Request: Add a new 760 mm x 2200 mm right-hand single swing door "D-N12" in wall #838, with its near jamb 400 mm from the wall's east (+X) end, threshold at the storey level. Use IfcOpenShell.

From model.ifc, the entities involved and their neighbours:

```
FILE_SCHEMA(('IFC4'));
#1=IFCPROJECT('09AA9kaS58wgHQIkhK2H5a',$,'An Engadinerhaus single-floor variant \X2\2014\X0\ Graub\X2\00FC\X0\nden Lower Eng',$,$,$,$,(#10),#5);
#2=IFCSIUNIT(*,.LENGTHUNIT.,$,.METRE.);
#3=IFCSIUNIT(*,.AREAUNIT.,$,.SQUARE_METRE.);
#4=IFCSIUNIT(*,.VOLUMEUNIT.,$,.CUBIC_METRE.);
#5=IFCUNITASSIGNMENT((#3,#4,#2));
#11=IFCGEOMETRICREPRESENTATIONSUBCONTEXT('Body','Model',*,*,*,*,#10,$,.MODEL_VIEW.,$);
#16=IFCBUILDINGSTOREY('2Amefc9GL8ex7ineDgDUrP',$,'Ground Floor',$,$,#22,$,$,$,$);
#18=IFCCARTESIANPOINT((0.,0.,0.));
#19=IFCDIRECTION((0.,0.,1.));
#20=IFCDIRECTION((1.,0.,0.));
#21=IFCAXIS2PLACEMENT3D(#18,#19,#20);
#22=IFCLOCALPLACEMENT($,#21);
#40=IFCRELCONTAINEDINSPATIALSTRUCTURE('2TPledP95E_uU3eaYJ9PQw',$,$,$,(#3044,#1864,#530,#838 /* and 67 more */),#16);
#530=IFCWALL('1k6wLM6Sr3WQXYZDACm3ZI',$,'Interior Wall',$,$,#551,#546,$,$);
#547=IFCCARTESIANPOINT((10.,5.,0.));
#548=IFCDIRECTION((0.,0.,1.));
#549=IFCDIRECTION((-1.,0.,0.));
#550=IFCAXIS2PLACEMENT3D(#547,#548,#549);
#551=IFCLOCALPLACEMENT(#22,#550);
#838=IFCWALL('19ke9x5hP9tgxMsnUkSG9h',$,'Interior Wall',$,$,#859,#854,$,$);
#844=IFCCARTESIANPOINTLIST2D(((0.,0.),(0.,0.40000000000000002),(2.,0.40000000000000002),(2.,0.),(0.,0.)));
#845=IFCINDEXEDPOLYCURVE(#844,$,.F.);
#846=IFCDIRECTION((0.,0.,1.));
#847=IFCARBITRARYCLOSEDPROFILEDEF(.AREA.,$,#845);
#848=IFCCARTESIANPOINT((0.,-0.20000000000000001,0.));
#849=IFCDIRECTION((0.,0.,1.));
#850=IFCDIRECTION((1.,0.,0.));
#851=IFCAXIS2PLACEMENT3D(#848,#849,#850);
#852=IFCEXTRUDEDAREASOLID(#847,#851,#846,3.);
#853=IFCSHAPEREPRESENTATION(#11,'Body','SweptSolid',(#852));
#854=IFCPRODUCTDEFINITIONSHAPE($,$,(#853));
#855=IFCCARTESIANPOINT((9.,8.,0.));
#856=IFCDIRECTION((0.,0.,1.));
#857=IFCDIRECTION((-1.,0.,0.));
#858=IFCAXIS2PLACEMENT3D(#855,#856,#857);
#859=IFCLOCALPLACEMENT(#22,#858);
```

```python
import numpy as np
import ifcopenshell
import ifcopenshell.api.feature
import ifcopenshell.api.geometry
import ifcopenshell.api.root
import ifcopenshell.api.spatial
import ifcopenshell.geom
import ifcopenshell.util.element
import ifcopenshell.util.placement
import ifcopenshell.util.representation
import ifcopenshell.util.shape
import ifcopenshell.util.unit

model = ifcopenshell.open("model.ifc")
unit_scale = ifcopenshell.util.unit.calculate_unit_scale(model)
settings = ifcopenshell.geom.settings()


def volume(element):
    """Net volume in cubic metres, openings subtracted."""
    shape = ifcopenshell.geom.create_shape(settings, element)
    return ifcopenshell.util.shape.get_volume(shape.geometry)


wall = model.by_guid("19ke9x5hP9tgxMsnUkSG9h")
storey = ifcopenshell.util.element.get_container(wall, ifc_class="IfcBuildingStorey")
context = ifcopenshell.util.representation.get_context(model, "Model", "Body", "MODEL_VIEW")
before = volume(wall)

width, height, from_end, sill = 0.76, 2.2, 0.4, 0.0  # metres

# The wall runs along its own X axis, and the end named is its -X end.
wall_shape = ifcopenshell.geom.create_shape(settings, wall)
x, y, z = ifcopenshell.util.shape.get_vertices(wall_shape.geometry).T
start = x.min() + from_end
face, thickness = float(y.min()), float(y.max() - y.min())
wall_matrix = ifcopenshell.util.placement.get_local_placement(wall.ObjectPlacement)
level = ifcopenshell.util.placement.get_local_placement(storey.ObjectPlacement)[2, 3]


def in_wall(x, y):
    """Placement at x, y metres in the wall's axes, at sill height."""
    matrix = wall_matrix.copy()
    matrix[:, 3] = wall_matrix @ np.array([x / unit_scale, y / unit_scale, 0.0, 1.0])
    matrix[2, 3] = level + sill / unit_scale
    return matrix


# Opening: a box that overshoots both wall faces by 50 mm.
opening = ifcopenshell.api.root.create_entity(model, ifc_class="IfcOpeningElement", predefined_type="OPENING")
box = ifcopenshell.api.geometry.add_wall_representation(
    model, context=context, length=width, height=height, thickness=thickness + 0.1
)
ifcopenshell.api.geometry.assign_representation(model, product=opening, representation=box)
ifcopenshell.api.geometry.edit_object_placement(model, product=opening, matrix=in_wall(start, face - 0.05), is_si=False)
ifcopenshell.api.feature.add_feature(model, feature=opening, element=wall)

door = ifcopenshell.api.root.create_entity(model, ifc_class="IfcDoor", name="D-N12", predefined_type="DOOR")
door.OverallWidth, door.OverallHeight = width / unit_scale, height / unit_scale
door.OperationType = "SINGLE_SWING_RIGHT"
body = ifcopenshell.api.geometry.add_door_representation(
    model,
    context=context,
    overall_width=door.OverallWidth,
    overall_height=door.OverallHeight,
    operation_type="SINGLE_SWING_RIGHT",
    lining_properties={"LiningDepth": thickness / unit_scale, "ThresholdDepth": thickness / unit_scale},
)
ifcopenshell.api.geometry.assign_representation(model, product=door, representation=body)
ifcopenshell.api.spatial.assign_container(model, products=[door], relating_structure=storey)
ifcopenshell.api.feature.add_filling(model, opening=opening, element=door)

# The lining spans the wall, so the door starts at the wall face.
ifcopenshell.api.geometry.edit_object_placement(model, product=door, matrix=in_wall(start, face), is_si=False)

after = volume(wall)

print(f"wall volume {before:.3f} -> {after:.3f} m3")

model.write("model_rev.ifc")
```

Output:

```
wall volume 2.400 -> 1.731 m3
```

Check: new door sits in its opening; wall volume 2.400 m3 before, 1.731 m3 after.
